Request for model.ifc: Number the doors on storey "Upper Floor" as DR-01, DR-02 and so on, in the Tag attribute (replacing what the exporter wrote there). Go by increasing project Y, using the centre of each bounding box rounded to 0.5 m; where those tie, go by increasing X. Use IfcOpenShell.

First a look at what the model holds.

```python
import ifcopenshell
import ifcopenshell.util.element
import ifcopenshell.util.placement

model = ifcopenshell.open("model.ifc")
print(model.schema)
storey = next(s for s in model.by_type("IfcBuildingStorey") if s.Name == "Upper Floor")
doors = [e for e in ifcopenshell.util.element.get_decomposition(storey) if e.is_a("IfcDoor")]
for e in sorted(doors, key=lambda e: e.id()):
    origin = ifcopenshell.util.placement.get_local_placement(e.ObjectPlacement)[:3, 3]
    print(e.id(), e.Tag, e.Name, origin.round(2) + 0.0, sep=" | ")
```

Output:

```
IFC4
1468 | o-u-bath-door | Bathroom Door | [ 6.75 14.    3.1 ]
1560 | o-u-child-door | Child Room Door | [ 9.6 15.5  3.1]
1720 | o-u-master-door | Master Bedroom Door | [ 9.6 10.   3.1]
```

```python
import ifcopenshell
import ifcopenshell.geom
import ifcopenshell.util.element
import ifcopenshell.util.shape

model = ifcopenshell.open("model.ifc")
settings = ifcopenshell.geom.settings()
settings.set("use-world-coords", True)


def centre(element):
    shape = ifcopenshell.geom.create_shape(settings, element)
    return ifcopenshell.util.shape.get_bbox_centroid(shape.geometry)


storey = next(s for s in model.by_type("IfcBuildingStorey") if s.Name == "Upper Floor")
doors = [e for e in ifcopenshell.util.element.get_decomposition(storey) if e.is_a("IfcDoor")]

# Insertion points can sit at a corner or the storey origin, so sort by the geometry (in metres).
centres = {e: centre(e) for e in doors}
doors.sort(key=lambda e: (round(centres[e][1] / 0.5), centres[e][0]))

for i, e in enumerate(doors, start=1):
    number = f"DR-{i:02d}"
    e.Tag = number
    print(e.id(), number)

model.write("model_updated.ifc")
```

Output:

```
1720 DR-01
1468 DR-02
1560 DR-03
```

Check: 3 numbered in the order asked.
